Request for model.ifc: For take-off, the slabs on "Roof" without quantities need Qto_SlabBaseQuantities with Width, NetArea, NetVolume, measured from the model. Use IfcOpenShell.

First a look at what the model holds.

```python
import ifcopenshell
import ifcopenshell.util.element
import ifcopenshell.util.unit

model = ifcopenshell.open("model.ifc")
print(model.schema)
for unit_type in ("LENGTHUNIT", "AREAUNIT", "VOLUMEUNIT"):
    print(unit_type, ifcopenshell.util.unit.calculate_unit_scale(model, unit_type))
storey = next(s for s in model.by_type("IfcBuildingStorey") if s.Name == "Roof")
slabs = [e for e in ifcopenshell.util.element.get_decomposition(storey) if e.is_a("IfcSlab")]
for e in sorted(slabs, key=lambda e: e.id()):
    print(e.id(), e.is_a(), e.Name, list(ifcopenshell.util.element.get_psets(e, qtos_only=True)), sep=" | ")
```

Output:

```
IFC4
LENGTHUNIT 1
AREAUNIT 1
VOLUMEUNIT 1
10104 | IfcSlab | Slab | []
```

```python
import ifcopenshell
import ifcopenshell.api.pset
import ifcopenshell.geom
import ifcopenshell.util.element
import ifcopenshell.util.shape
import ifcopenshell.util.unit

model = ifcopenshell.open("model.ifc")
unit_scale = ifcopenshell.util.unit.calculate_unit_scale(model)
area_scale = ifcopenshell.util.unit.calculate_unit_scale(model, "AREAUNIT")
volume_scale = ifcopenshell.util.unit.calculate_unit_scale(model, "VOLUMEUNIT")
settings = ifcopenshell.geom.settings()

storey = next(s for s in model.by_type("IfcBuildingStorey") if s.Name == "Roof")
slabs = [e for e in ifcopenshell.util.element.get_decomposition(storey) if e.is_a("IfcSlab")]

for e in sorted(slabs, key=lambda e: e.id()):
    if ifcopenshell.util.element.get_psets(e, qtos_only=True, should_inherit=False):
        continue
    # Geometry comes back in metres, in the element's own axes.
    shape = ifcopenshell.geom.create_shape(settings, e)
    values = {
        "Width": ifcopenshell.util.shape.get_z(shape.geometry) / unit_scale,
        "NetArea": ifcopenshell.util.shape.get_footprint_area(shape.geometry) / area_scale,
        "NetVolume": ifcopenshell.util.shape.get_volume(shape.geometry) / volume_scale,
    }
    qto = ifcopenshell.api.pset.add_qto(model, product=e, name="Qto_SlabBaseQuantities")
    ifcopenshell.api.pset.edit_qto(model, qto=qto, properties=values)
    print(e.id(), {k: round(v, 3) for k, v in values.items()})

model.write("model_updated.ifc")
```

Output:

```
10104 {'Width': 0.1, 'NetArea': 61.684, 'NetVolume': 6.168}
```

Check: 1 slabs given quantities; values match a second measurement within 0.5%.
